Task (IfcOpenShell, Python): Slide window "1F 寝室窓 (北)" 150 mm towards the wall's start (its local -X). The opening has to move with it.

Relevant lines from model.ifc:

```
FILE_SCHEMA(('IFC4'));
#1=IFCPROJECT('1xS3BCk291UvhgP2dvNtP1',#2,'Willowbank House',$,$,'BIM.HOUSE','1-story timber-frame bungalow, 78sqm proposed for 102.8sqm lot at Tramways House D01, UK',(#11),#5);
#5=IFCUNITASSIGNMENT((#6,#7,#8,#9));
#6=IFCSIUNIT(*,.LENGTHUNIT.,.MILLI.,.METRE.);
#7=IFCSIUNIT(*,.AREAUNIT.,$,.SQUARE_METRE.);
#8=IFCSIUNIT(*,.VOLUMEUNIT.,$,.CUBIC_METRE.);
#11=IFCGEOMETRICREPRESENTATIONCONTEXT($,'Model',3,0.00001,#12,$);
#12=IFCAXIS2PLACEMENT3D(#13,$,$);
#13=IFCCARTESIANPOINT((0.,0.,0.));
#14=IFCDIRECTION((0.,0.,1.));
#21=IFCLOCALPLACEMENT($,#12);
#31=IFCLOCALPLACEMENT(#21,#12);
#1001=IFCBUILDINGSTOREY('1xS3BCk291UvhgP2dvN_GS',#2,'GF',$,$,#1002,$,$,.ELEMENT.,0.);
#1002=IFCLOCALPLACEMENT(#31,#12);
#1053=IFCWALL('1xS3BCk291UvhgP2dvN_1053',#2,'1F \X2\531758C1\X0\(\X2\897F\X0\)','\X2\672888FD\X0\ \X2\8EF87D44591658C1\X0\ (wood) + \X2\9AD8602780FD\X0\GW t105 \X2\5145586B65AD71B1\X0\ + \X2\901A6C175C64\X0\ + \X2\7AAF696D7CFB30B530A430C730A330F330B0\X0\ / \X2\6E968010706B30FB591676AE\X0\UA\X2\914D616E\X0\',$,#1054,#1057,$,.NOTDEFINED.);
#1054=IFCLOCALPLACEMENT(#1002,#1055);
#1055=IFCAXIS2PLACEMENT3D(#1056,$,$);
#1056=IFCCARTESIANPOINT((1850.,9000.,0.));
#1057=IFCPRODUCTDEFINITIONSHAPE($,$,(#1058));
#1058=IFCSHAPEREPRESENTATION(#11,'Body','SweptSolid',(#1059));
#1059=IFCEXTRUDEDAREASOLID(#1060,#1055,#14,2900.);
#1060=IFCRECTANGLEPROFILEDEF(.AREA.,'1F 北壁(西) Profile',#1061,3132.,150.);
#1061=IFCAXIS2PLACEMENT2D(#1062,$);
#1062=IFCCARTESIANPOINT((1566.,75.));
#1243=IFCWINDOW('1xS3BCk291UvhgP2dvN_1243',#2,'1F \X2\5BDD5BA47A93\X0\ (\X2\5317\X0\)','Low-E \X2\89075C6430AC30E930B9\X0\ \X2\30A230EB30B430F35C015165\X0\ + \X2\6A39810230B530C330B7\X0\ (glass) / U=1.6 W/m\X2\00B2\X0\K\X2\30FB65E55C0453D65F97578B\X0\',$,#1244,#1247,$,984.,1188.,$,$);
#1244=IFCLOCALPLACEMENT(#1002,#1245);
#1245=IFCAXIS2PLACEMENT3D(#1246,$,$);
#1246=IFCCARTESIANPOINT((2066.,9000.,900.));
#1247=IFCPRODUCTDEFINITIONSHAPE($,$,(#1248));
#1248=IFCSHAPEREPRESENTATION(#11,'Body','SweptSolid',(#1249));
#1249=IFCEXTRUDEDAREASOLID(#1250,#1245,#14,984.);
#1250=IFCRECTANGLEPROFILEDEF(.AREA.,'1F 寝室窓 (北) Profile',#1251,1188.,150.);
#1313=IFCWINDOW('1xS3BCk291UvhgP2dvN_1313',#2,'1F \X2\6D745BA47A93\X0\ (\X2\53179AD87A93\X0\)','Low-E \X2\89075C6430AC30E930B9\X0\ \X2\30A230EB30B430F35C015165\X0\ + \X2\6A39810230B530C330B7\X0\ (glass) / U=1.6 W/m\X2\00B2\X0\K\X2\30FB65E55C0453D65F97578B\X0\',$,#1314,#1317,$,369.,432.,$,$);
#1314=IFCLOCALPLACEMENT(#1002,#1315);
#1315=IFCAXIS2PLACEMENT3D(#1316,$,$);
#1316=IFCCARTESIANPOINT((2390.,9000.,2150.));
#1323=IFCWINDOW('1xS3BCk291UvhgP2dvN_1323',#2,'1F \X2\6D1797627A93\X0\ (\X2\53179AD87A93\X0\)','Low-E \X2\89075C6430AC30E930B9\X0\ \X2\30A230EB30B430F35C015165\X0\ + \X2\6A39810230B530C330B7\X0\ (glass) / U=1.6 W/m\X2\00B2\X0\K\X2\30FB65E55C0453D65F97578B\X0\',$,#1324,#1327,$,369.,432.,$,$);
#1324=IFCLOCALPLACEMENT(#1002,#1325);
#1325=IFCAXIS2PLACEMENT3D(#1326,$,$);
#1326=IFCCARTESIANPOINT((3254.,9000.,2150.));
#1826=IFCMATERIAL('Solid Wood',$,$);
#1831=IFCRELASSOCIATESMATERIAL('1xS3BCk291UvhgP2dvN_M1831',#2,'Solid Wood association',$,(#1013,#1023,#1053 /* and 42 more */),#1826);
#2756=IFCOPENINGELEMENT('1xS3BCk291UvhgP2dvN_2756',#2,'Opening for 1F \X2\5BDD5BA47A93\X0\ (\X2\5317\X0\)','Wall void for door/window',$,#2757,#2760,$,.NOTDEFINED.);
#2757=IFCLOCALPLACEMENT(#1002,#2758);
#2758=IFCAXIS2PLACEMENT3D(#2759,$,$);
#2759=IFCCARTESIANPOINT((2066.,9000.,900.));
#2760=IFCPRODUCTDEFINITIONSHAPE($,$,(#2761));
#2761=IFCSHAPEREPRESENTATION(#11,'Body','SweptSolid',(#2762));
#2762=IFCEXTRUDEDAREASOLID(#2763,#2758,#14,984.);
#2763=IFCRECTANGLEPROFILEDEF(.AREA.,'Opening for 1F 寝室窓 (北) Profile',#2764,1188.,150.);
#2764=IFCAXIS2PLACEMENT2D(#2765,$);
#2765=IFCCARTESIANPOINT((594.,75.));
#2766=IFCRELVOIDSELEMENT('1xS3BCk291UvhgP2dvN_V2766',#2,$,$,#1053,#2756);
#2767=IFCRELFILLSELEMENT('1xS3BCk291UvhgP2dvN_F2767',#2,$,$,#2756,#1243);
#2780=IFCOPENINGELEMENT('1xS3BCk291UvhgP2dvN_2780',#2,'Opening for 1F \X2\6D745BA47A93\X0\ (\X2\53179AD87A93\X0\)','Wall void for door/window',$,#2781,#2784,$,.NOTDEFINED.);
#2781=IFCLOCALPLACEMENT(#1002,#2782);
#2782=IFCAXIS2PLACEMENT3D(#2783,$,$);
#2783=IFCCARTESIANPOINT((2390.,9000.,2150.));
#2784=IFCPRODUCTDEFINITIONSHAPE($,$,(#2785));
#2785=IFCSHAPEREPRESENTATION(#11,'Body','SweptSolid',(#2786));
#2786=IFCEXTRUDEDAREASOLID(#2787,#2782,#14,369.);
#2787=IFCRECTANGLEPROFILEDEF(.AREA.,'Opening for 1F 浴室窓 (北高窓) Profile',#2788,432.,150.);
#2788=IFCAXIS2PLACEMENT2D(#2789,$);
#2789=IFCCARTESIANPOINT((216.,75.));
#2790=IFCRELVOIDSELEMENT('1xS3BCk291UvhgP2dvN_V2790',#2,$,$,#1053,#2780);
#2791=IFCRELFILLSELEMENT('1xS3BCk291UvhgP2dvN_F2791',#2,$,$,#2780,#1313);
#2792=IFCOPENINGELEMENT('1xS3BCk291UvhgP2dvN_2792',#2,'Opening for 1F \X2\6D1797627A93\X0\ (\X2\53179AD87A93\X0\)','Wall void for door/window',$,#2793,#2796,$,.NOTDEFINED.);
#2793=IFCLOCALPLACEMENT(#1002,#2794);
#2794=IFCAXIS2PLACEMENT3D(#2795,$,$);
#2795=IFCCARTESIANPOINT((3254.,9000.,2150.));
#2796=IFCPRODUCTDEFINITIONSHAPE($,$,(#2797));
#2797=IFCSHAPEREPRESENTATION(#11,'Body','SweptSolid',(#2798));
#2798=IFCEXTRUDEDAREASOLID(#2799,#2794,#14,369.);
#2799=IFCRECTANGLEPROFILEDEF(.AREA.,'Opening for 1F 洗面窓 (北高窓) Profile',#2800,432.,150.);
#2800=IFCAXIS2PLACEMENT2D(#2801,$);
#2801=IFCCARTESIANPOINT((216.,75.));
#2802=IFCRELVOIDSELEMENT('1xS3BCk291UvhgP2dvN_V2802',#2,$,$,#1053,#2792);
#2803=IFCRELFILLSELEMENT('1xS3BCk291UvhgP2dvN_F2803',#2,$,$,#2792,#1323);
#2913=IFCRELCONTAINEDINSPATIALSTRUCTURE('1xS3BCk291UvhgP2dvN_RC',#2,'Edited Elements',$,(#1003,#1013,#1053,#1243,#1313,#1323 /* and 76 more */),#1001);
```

```python
import ifcopenshell
import ifcopenshell.api.geometry
import ifcopenshell.util.placement
import ifcopenshell.util.unit

model = ifcopenshell.open("model.ifc")
unit_scale = ifcopenshell.util.unit.calculate_unit_scale(model)

window = model.by_id(1243)
opening = window.FillsVoids[0].RelatingOpeningElement
wall = opening.VoidsElements[0].RelatingBuildingElement

wall_matrix = ifcopenshell.util.placement.get_local_placement(wall.ObjectPlacement)
shift = wall_matrix[:3, 0] * -0.15 / unit_scale
before = ifcopenshell.util.placement.get_local_placement(window.ObjectPlacement)[:3, 3].copy()

# The window is not placed relative to its opening, so move both.
for product in (opening, window):
    matrix = ifcopenshell.util.placement.get_local_placement(product.ObjectPlacement)
    matrix[:3, 3] += shift
    ifcopenshell.api.geometry.edit_object_placement(model, product=product, matrix=matrix, is_si=False)

after = ifcopenshell.util.placement.get_local_placement(window.ObjectPlacement)[:3, 3]
print("window moved by", (after - before).round(3) + 0.0)

model.write("model_v2.ifc")
```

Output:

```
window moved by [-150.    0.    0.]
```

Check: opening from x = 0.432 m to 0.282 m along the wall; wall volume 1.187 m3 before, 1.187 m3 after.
